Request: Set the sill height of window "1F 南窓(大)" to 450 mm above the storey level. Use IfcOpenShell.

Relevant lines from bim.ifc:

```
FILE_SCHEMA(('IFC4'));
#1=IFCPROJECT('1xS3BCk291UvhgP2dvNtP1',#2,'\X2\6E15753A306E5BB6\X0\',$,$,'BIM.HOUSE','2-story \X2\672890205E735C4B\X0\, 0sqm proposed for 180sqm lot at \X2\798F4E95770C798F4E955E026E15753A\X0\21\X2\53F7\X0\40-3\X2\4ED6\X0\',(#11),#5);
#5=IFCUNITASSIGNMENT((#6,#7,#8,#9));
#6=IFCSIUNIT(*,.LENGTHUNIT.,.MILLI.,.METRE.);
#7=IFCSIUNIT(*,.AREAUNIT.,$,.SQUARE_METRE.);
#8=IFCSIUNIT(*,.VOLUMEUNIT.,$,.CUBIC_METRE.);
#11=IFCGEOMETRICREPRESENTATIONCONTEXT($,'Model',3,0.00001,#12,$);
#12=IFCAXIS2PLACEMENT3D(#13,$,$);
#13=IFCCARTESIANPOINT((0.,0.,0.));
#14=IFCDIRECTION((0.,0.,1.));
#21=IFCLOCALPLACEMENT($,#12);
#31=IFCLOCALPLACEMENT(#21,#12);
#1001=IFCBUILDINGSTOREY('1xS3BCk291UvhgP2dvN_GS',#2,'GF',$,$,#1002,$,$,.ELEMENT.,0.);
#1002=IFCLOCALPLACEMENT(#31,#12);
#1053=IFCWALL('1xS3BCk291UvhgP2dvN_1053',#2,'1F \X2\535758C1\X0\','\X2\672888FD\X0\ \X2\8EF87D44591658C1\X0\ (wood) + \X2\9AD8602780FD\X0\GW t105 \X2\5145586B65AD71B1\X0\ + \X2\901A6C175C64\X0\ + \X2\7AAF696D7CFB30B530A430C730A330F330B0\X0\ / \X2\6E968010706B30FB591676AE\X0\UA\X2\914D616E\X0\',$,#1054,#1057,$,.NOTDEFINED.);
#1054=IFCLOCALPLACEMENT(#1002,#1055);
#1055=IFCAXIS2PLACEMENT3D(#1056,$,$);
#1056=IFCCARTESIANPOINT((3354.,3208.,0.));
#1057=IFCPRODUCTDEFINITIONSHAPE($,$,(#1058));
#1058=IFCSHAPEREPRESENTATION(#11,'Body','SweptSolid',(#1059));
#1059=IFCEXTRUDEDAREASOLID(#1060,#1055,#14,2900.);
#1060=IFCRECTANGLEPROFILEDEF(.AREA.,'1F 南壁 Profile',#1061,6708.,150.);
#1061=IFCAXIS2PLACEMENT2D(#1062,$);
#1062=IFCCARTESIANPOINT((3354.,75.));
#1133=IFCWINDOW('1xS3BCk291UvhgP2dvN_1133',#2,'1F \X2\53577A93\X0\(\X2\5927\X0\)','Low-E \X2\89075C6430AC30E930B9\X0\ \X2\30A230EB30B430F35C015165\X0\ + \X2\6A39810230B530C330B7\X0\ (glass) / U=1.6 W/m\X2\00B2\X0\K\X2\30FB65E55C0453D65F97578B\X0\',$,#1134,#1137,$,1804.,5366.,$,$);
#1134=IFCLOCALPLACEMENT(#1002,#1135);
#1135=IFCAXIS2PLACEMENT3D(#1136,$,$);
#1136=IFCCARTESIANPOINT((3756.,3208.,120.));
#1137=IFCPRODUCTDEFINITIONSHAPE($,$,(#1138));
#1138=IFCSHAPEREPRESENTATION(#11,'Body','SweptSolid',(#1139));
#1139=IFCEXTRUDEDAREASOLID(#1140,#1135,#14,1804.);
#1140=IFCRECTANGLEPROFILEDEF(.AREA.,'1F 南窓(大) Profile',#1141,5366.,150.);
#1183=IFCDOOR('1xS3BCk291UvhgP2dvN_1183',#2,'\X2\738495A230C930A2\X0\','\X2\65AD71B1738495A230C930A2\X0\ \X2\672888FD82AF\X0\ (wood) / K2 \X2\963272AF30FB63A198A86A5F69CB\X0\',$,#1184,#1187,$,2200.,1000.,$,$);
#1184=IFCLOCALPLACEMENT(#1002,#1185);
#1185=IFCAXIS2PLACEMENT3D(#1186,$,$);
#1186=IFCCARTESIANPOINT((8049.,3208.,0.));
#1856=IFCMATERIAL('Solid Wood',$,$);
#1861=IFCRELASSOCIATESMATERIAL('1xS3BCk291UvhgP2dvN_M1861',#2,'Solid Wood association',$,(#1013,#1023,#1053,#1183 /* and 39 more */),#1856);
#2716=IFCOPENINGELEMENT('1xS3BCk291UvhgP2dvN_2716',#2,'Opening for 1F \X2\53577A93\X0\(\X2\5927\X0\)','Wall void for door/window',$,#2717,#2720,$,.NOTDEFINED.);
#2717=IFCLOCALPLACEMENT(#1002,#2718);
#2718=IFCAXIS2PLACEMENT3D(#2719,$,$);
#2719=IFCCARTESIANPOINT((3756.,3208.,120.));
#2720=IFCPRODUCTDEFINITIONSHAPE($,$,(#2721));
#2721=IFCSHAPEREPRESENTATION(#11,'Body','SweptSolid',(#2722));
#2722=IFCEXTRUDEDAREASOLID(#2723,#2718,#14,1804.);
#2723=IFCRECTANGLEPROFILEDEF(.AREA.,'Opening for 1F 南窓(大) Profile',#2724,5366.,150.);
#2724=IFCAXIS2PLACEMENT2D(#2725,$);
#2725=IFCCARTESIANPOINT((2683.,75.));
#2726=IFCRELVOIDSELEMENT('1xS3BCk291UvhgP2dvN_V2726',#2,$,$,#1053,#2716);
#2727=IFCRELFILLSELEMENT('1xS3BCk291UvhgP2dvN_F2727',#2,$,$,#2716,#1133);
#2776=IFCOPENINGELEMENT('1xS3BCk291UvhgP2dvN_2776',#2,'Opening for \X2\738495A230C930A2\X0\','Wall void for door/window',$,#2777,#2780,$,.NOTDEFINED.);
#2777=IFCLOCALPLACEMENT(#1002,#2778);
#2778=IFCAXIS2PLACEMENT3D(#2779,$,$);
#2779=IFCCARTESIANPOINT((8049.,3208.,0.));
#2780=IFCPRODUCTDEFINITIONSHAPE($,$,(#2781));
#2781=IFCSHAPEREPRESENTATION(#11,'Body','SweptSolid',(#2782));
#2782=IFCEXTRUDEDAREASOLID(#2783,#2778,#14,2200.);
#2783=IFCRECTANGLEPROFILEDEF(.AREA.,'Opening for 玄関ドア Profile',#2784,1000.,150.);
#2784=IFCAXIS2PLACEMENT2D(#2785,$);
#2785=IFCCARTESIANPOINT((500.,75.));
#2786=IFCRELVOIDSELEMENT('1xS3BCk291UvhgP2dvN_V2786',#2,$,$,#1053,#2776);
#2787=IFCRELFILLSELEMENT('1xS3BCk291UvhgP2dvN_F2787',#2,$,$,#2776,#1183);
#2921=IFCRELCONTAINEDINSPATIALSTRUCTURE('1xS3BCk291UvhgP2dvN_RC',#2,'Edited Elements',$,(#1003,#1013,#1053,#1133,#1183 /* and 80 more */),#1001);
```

```python
import numpy as np
import ifcopenshell
import ifcopenshell.api.geometry
import ifcopenshell.geom
import ifcopenshell.util.element
import ifcopenshell.util.placement
import ifcopenshell.util.shape
import ifcopenshell.util.unit

model = ifcopenshell.open("bim.ifc")
unit_scale = ifcopenshell.util.unit.calculate_unit_scale(model)

window = model.by_guid("1xS3BCk291UvhgP2dvN_1133")
opening = window.FillsVoids[0].RelatingOpeningElement
storey = ifcopenshell.util.element.get_container(window, ifc_class="IfcBuildingStorey")
level = ifcopenshell.util.placement.get_local_placement(storey.ObjectPlacement)[2, 3]

# The opening's origin need not be at the sill, so measure its lowest point.
shape = ifcopenshell.geom.create_shape(ifcopenshell.geom.settings(), opening)
bottom = ifcopenshell.util.shape.get_shape_bottom_elevation(shape, shape.geometry) / unit_scale
dz = level + 450.0 - bottom

shift = np.array([0.0, 0.0, dz])
# The window is not placed relative to its opening, so move both.
for product in (opening, window):
    matrix = ifcopenshell.util.placement.get_local_placement(product.ObjectPlacement)
    matrix[:3, 3] += shift
    ifcopenshell.api.geometry.edit_object_placement(model, product=product, matrix=matrix, is_si=False)

print(f"moved by {dz * unit_scale:+.3f} m")

model.write("bim_v2.ifc")
```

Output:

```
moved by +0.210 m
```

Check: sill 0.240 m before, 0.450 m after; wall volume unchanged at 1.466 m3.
